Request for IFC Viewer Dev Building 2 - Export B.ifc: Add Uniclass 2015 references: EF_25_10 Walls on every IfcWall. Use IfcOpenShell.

First a look at what the model holds.

```python
import ifcopenshell

model = ifcopenshell.open("IFC Viewer Dev Building 2 - Export B.ifc")
print(model.schema)
print("classifications:", [c.Name for c in model.by_type("IfcClassification")])
for ifc_class in ("IfcDoor", "IfcRoof", "IfcStair", "IfcWall", "IfcWindow"):
    print(ifc_class, len(model.by_type(ifc_class)))
```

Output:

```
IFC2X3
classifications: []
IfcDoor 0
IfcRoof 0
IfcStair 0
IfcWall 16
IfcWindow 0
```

```python
import ifcopenshell
import ifcopenshell.api.classification

model = ifcopenshell.open("IFC Viewer Dev Building 2 - Export B.ifc")

# IFC2X3 requires Source and Edition and has no link from the project to the system.
system = model.create_entity("IfcClassification", Source="NBS", Edition="2015", Name="Uniclass 2015")

codes = {
    "IfcWall": ("EF_25_10", "Walls"),
}
for ifc_class, (code, name) in codes.items():
    products = model.by_type(ifc_class)
    ifcopenshell.api.classification.add_reference(
        model, products=products, classification=system, identification=code, name=name
    )
    print(code, len(products))

model.write("IFC Viewer Dev Building 2 - Export B_edited.ifc")
```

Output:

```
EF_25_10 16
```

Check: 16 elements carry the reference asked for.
